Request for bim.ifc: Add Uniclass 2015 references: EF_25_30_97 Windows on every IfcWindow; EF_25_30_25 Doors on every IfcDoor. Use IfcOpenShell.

First a look at what the model holds.

```python
import ifcopenshell

model = ifcopenshell.open("bim.ifc")
print(model.schema)
print("classifications:", [c.Name for c in model.by_type("IfcClassification")])
for ifc_class in ("IfcDoor", "IfcRoof", "IfcStair", "IfcWall", "IfcWindow"):
    print(ifc_class, len(model.by_type(ifc_class)))
```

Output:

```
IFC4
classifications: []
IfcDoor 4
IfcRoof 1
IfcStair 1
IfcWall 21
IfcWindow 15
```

```python
import ifcopenshell
import ifcopenshell.api.classification

model = ifcopenshell.open("bim.ifc")

system = ifcopenshell.api.classification.add_classification(model, classification="Uniclass 2015")

codes = {
    "IfcWindow": ("EF_25_30_97", "Windows"),
    "IfcDoor": ("EF_25_30_25", "Doors"),
}
for ifc_class, (code, name) in codes.items():
    products = model.by_type(ifc_class)
    ifcopenshell.api.classification.add_reference(
        model, products=products, classification=system, identification=code, name=name
    )
    print(code, len(products))

model.write("bim-out.ifc")
```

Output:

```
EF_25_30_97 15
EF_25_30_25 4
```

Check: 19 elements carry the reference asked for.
